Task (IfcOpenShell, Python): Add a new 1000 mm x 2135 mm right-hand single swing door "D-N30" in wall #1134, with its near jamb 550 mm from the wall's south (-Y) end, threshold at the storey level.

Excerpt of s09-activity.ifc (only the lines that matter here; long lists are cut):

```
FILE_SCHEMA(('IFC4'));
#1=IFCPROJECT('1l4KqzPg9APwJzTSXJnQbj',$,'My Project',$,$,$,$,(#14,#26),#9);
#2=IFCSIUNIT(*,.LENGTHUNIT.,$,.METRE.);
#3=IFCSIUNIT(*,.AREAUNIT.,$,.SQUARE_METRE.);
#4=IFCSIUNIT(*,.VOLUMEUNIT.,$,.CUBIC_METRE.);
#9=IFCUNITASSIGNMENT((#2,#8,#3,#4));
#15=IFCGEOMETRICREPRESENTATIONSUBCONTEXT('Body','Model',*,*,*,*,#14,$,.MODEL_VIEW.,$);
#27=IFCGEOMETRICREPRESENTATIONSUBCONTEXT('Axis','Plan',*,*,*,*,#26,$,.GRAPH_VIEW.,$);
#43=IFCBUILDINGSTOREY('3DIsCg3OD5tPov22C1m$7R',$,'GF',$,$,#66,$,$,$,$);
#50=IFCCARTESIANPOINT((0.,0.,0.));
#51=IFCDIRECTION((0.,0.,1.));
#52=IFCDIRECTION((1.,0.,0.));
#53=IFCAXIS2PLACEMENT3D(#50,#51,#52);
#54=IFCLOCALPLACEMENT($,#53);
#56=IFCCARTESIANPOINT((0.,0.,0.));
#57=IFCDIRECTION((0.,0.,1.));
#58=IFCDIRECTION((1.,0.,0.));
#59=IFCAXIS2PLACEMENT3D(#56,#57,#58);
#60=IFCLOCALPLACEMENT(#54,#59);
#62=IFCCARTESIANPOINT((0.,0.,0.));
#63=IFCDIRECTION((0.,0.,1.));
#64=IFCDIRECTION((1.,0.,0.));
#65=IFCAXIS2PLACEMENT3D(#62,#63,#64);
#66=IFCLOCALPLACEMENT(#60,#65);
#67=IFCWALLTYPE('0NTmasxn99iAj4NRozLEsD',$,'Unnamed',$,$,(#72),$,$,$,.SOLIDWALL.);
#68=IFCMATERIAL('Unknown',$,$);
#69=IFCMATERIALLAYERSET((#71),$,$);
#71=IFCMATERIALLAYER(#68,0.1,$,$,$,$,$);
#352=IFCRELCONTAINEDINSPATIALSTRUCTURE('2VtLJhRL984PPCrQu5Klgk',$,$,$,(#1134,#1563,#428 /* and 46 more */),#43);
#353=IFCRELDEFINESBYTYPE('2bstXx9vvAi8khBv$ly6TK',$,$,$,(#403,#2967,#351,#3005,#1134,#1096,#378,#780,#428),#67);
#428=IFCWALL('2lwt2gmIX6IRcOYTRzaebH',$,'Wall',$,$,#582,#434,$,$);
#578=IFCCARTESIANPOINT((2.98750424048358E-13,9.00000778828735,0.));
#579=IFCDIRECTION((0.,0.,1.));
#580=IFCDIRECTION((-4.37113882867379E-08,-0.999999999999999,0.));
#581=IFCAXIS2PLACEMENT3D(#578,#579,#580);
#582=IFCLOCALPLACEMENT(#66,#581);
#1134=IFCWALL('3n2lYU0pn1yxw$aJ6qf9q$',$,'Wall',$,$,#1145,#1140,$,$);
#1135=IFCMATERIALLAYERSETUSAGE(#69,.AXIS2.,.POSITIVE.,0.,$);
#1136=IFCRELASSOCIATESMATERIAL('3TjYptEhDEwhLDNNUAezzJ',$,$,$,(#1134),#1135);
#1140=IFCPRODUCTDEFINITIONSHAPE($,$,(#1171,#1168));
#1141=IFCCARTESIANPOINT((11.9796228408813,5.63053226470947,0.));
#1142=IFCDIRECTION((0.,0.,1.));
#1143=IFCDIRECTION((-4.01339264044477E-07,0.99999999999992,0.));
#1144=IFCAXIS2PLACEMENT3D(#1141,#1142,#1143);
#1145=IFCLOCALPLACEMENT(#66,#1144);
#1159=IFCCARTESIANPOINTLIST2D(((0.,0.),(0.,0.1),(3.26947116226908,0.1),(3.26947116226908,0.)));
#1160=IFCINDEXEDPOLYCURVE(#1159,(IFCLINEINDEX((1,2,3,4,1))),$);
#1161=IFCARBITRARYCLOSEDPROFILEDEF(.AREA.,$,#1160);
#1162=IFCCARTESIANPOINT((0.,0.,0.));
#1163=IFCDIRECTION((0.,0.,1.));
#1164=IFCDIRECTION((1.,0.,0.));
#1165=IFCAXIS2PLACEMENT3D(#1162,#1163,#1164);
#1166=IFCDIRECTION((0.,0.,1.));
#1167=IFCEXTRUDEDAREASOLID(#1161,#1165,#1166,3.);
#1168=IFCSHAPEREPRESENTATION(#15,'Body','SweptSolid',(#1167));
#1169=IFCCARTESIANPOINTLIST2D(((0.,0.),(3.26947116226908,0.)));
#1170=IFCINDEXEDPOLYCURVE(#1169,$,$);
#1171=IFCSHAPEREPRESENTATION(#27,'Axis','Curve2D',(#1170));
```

```python
import numpy as np
import ifcopenshell
import ifcopenshell.api.feature
import ifcopenshell.api.geometry
import ifcopenshell.api.root
import ifcopenshell.api.spatial
import ifcopenshell.geom
import ifcopenshell.util.element
import ifcopenshell.util.placement
import ifcopenshell.util.representation
import ifcopenshell.util.shape
import ifcopenshell.util.unit

model = ifcopenshell.open("s09-activity.ifc")
unit_scale = ifcopenshell.util.unit.calculate_unit_scale(model)
settings = ifcopenshell.geom.settings()


def volume(element):
    """Net volume in cubic metres, openings subtracted."""
    shape = ifcopenshell.geom.create_shape(settings, element)
    return ifcopenshell.util.shape.get_volume(shape.geometry)


wall = model.by_id(1134)
storey = ifcopenshell.util.element.get_container(wall, ifc_class="IfcBuildingStorey")
context = ifcopenshell.util.representation.get_context(model, "Model", "Body", "MODEL_VIEW")
before = volume(wall)

width, height, from_end, sill = 1, 2.135, 0.55, 0.0  # metres

# The wall runs along its own X axis, and the end named is its -X end.
wall_shape = ifcopenshell.geom.create_shape(settings, wall)
x, y, z = ifcopenshell.util.shape.get_vertices(wall_shape.geometry).T
start = x.min() + from_end
face, thickness = float(y.min()), float(y.max() - y.min())
wall_matrix = ifcopenshell.util.placement.get_local_placement(wall.ObjectPlacement)
level = ifcopenshell.util.placement.get_local_placement(storey.ObjectPlacement)[2, 3]


def in_wall(x, y):
    """Placement at x, y metres in the wall's axes, at sill height."""
    matrix = wall_matrix.copy()
    matrix[:, 3] = wall_matrix @ np.array([x / unit_scale, y / unit_scale, 0.0, 1.0])
    matrix[2, 3] = level + sill / unit_scale
    return matrix


# Opening: a box that overshoots both wall faces by 50 mm.
opening = ifcopenshell.api.root.create_entity(model, ifc_class="IfcOpeningElement", predefined_type="OPENING")
box = ifcopenshell.api.geometry.add_wall_representation(
    model, context=context, length=width, height=height, thickness=thickness + 0.1
)
ifcopenshell.api.geometry.assign_representation(model, product=opening, representation=box)
ifcopenshell.api.geometry.edit_object_placement(model, product=opening, matrix=in_wall(start, face - 0.05), is_si=False)
ifcopenshell.api.feature.add_feature(model, feature=opening, element=wall)

door = ifcopenshell.api.root.create_entity(model, ifc_class="IfcDoor", name="D-N30", predefined_type="DOOR")
door.OverallWidth, door.OverallHeight = width / unit_scale, height / unit_scale
door.OperationType = "SINGLE_SWING_RIGHT"
body = ifcopenshell.api.geometry.add_door_representation(
    model,
    context=context,
    overall_width=door.OverallWidth,
    overall_height=door.OverallHeight,
    operation_type="SINGLE_SWING_RIGHT",
    lining_properties={"LiningDepth": thickness / unit_scale, "ThresholdDepth": thickness / unit_scale},
)
ifcopenshell.api.geometry.assign_representation(model, product=door, representation=body)
ifcopenshell.api.spatial.assign_container(model, products=[door], relating_structure=storey)
ifcopenshell.api.feature.add_filling(model, opening=opening, element=door)

# The lining spans the wall, so the door starts at the wall face.
ifcopenshell.api.geometry.edit_object_placement(model, product=door, matrix=in_wall(start, face), is_si=False)

after = volume(wall)

print(f"wall volume {before:.3f} -> {after:.3f} m3")

model.write("s09-activity_v2.ifc")
```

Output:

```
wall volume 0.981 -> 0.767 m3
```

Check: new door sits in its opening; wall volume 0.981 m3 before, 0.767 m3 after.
